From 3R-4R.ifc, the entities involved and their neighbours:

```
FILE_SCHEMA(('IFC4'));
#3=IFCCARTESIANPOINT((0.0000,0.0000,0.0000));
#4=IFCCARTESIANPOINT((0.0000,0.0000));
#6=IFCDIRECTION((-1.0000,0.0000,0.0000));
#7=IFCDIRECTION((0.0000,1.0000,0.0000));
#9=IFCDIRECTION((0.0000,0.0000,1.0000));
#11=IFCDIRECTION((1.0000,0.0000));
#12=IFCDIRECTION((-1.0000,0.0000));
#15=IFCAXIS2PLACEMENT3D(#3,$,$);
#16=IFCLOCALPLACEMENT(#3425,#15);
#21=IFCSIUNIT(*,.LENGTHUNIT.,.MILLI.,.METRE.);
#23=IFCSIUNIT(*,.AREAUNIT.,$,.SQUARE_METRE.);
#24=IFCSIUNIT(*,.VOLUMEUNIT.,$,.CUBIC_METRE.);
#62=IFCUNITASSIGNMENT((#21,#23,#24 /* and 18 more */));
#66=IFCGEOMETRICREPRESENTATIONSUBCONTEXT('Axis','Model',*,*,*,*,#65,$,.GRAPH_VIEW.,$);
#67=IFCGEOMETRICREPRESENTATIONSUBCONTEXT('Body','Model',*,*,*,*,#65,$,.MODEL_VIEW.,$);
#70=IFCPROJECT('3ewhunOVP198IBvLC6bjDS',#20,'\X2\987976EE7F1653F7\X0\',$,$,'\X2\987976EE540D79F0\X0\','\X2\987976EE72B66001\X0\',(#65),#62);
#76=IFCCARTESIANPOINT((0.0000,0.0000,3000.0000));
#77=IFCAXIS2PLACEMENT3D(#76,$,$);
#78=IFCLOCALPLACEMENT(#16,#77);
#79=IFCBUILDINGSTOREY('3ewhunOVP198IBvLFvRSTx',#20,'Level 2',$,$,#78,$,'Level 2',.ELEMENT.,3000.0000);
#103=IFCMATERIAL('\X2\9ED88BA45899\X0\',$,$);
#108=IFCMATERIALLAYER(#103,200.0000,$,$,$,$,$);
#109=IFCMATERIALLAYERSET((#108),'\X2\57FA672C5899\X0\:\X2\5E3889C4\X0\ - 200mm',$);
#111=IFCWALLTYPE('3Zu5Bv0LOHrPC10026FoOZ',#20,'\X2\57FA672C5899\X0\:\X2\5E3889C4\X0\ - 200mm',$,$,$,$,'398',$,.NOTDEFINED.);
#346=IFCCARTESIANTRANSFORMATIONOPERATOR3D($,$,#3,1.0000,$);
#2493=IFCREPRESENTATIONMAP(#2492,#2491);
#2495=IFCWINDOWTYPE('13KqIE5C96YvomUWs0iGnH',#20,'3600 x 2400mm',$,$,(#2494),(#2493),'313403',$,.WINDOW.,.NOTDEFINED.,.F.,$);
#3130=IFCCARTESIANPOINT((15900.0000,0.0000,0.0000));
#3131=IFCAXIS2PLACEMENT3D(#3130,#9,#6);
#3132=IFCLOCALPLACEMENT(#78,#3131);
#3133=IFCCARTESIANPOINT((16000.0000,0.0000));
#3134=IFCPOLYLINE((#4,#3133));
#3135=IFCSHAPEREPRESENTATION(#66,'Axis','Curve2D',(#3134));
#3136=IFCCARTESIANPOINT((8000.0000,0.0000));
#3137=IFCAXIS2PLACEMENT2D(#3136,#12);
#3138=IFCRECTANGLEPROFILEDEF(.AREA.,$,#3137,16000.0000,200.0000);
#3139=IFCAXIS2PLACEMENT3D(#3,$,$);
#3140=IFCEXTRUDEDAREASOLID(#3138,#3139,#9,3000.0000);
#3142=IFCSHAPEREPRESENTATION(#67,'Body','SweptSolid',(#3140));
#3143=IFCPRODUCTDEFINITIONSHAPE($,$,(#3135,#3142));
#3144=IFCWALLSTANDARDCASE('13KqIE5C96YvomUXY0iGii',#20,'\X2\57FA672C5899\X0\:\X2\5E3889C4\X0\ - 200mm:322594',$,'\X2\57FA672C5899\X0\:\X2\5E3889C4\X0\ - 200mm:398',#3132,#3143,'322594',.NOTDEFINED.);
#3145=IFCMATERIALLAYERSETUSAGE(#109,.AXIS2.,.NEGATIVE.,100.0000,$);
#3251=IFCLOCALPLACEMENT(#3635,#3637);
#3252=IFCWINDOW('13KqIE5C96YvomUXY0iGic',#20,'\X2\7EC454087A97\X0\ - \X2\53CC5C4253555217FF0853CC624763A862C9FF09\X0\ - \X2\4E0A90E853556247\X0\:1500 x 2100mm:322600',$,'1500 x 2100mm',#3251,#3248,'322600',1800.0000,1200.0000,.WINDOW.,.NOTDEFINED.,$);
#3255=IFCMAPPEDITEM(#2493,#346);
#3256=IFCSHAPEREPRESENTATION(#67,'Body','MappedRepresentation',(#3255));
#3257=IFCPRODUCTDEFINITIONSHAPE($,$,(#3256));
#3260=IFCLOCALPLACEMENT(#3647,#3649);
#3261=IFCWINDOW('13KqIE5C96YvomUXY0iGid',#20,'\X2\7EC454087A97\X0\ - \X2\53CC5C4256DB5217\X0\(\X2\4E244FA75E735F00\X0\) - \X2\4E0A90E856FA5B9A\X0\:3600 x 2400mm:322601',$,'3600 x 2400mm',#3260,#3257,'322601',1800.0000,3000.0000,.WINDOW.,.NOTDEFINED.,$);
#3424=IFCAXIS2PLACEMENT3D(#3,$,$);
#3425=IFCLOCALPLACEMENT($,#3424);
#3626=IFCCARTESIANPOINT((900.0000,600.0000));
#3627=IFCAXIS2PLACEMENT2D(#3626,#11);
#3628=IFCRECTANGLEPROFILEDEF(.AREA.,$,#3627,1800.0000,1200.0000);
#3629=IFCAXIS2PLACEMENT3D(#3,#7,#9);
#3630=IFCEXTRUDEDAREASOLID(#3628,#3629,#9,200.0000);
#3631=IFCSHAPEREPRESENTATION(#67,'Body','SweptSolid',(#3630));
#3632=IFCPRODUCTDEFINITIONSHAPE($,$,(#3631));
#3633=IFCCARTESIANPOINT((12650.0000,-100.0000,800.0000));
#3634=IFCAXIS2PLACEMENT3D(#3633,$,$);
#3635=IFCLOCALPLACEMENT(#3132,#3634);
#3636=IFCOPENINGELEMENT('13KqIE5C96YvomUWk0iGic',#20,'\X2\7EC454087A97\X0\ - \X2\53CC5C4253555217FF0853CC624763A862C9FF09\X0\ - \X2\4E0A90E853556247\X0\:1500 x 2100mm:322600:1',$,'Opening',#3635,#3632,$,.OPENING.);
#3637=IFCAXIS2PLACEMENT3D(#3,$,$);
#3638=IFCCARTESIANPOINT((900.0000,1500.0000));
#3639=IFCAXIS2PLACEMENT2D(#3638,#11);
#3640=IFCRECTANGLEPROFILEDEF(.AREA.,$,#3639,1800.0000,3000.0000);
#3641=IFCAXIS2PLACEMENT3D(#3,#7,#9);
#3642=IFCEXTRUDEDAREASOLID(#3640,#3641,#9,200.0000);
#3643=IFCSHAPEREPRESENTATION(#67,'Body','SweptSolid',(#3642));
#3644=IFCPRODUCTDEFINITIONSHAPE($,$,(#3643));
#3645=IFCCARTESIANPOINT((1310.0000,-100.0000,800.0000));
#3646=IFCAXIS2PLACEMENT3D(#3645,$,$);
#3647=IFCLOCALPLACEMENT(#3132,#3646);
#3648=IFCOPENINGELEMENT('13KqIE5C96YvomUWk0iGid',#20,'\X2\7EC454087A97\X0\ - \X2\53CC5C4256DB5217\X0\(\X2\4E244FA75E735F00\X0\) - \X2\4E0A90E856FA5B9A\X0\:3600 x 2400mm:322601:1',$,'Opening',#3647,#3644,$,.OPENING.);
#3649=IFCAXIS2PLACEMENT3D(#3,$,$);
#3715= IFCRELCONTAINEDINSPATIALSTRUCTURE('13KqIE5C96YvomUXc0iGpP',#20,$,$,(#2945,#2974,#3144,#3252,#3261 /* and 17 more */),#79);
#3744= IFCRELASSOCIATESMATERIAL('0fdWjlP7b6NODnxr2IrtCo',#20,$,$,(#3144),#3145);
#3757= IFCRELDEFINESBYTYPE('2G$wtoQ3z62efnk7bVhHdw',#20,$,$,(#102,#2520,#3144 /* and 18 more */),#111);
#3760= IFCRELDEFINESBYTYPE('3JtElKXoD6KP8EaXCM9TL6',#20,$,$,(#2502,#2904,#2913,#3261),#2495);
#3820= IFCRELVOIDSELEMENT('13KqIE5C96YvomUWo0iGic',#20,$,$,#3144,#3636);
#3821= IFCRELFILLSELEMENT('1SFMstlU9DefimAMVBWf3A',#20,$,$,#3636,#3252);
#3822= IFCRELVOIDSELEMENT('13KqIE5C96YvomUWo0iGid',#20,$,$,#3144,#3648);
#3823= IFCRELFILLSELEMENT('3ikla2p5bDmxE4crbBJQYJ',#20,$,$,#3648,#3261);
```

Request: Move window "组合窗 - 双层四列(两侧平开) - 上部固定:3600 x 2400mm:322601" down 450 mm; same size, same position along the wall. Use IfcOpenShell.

```python
import numpy as np
import ifcopenshell
import ifcopenshell.api.geometry
import ifcopenshell.util.placement
import ifcopenshell.util.unit

model = ifcopenshell.open("3R-4R.ifc")
unit_scale = ifcopenshell.util.unit.calculate_unit_scale(model)

window = model.by_guid("13KqIE5C96YvomUXY0iGid")
opening = window.FillsVoids[0].RelatingOpeningElement
dz = -0.45 / unit_scale

shift = np.array([0.0, 0.0, dz])
# The window is placed relative to its opening, so it follows when the opening moves.
matrix = ifcopenshell.util.placement.get_local_placement(opening.ObjectPlacement)
matrix[:3, 3] += shift
ifcopenshell.api.geometry.edit_object_placement(
    model, product=opening, matrix=matrix, is_si=False, should_transform_children=True
)

print(f"moved by {dz * unit_scale:+.3f} m")

model.write("3R-4R_edited.ifc")
```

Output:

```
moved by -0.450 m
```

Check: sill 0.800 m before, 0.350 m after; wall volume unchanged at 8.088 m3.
